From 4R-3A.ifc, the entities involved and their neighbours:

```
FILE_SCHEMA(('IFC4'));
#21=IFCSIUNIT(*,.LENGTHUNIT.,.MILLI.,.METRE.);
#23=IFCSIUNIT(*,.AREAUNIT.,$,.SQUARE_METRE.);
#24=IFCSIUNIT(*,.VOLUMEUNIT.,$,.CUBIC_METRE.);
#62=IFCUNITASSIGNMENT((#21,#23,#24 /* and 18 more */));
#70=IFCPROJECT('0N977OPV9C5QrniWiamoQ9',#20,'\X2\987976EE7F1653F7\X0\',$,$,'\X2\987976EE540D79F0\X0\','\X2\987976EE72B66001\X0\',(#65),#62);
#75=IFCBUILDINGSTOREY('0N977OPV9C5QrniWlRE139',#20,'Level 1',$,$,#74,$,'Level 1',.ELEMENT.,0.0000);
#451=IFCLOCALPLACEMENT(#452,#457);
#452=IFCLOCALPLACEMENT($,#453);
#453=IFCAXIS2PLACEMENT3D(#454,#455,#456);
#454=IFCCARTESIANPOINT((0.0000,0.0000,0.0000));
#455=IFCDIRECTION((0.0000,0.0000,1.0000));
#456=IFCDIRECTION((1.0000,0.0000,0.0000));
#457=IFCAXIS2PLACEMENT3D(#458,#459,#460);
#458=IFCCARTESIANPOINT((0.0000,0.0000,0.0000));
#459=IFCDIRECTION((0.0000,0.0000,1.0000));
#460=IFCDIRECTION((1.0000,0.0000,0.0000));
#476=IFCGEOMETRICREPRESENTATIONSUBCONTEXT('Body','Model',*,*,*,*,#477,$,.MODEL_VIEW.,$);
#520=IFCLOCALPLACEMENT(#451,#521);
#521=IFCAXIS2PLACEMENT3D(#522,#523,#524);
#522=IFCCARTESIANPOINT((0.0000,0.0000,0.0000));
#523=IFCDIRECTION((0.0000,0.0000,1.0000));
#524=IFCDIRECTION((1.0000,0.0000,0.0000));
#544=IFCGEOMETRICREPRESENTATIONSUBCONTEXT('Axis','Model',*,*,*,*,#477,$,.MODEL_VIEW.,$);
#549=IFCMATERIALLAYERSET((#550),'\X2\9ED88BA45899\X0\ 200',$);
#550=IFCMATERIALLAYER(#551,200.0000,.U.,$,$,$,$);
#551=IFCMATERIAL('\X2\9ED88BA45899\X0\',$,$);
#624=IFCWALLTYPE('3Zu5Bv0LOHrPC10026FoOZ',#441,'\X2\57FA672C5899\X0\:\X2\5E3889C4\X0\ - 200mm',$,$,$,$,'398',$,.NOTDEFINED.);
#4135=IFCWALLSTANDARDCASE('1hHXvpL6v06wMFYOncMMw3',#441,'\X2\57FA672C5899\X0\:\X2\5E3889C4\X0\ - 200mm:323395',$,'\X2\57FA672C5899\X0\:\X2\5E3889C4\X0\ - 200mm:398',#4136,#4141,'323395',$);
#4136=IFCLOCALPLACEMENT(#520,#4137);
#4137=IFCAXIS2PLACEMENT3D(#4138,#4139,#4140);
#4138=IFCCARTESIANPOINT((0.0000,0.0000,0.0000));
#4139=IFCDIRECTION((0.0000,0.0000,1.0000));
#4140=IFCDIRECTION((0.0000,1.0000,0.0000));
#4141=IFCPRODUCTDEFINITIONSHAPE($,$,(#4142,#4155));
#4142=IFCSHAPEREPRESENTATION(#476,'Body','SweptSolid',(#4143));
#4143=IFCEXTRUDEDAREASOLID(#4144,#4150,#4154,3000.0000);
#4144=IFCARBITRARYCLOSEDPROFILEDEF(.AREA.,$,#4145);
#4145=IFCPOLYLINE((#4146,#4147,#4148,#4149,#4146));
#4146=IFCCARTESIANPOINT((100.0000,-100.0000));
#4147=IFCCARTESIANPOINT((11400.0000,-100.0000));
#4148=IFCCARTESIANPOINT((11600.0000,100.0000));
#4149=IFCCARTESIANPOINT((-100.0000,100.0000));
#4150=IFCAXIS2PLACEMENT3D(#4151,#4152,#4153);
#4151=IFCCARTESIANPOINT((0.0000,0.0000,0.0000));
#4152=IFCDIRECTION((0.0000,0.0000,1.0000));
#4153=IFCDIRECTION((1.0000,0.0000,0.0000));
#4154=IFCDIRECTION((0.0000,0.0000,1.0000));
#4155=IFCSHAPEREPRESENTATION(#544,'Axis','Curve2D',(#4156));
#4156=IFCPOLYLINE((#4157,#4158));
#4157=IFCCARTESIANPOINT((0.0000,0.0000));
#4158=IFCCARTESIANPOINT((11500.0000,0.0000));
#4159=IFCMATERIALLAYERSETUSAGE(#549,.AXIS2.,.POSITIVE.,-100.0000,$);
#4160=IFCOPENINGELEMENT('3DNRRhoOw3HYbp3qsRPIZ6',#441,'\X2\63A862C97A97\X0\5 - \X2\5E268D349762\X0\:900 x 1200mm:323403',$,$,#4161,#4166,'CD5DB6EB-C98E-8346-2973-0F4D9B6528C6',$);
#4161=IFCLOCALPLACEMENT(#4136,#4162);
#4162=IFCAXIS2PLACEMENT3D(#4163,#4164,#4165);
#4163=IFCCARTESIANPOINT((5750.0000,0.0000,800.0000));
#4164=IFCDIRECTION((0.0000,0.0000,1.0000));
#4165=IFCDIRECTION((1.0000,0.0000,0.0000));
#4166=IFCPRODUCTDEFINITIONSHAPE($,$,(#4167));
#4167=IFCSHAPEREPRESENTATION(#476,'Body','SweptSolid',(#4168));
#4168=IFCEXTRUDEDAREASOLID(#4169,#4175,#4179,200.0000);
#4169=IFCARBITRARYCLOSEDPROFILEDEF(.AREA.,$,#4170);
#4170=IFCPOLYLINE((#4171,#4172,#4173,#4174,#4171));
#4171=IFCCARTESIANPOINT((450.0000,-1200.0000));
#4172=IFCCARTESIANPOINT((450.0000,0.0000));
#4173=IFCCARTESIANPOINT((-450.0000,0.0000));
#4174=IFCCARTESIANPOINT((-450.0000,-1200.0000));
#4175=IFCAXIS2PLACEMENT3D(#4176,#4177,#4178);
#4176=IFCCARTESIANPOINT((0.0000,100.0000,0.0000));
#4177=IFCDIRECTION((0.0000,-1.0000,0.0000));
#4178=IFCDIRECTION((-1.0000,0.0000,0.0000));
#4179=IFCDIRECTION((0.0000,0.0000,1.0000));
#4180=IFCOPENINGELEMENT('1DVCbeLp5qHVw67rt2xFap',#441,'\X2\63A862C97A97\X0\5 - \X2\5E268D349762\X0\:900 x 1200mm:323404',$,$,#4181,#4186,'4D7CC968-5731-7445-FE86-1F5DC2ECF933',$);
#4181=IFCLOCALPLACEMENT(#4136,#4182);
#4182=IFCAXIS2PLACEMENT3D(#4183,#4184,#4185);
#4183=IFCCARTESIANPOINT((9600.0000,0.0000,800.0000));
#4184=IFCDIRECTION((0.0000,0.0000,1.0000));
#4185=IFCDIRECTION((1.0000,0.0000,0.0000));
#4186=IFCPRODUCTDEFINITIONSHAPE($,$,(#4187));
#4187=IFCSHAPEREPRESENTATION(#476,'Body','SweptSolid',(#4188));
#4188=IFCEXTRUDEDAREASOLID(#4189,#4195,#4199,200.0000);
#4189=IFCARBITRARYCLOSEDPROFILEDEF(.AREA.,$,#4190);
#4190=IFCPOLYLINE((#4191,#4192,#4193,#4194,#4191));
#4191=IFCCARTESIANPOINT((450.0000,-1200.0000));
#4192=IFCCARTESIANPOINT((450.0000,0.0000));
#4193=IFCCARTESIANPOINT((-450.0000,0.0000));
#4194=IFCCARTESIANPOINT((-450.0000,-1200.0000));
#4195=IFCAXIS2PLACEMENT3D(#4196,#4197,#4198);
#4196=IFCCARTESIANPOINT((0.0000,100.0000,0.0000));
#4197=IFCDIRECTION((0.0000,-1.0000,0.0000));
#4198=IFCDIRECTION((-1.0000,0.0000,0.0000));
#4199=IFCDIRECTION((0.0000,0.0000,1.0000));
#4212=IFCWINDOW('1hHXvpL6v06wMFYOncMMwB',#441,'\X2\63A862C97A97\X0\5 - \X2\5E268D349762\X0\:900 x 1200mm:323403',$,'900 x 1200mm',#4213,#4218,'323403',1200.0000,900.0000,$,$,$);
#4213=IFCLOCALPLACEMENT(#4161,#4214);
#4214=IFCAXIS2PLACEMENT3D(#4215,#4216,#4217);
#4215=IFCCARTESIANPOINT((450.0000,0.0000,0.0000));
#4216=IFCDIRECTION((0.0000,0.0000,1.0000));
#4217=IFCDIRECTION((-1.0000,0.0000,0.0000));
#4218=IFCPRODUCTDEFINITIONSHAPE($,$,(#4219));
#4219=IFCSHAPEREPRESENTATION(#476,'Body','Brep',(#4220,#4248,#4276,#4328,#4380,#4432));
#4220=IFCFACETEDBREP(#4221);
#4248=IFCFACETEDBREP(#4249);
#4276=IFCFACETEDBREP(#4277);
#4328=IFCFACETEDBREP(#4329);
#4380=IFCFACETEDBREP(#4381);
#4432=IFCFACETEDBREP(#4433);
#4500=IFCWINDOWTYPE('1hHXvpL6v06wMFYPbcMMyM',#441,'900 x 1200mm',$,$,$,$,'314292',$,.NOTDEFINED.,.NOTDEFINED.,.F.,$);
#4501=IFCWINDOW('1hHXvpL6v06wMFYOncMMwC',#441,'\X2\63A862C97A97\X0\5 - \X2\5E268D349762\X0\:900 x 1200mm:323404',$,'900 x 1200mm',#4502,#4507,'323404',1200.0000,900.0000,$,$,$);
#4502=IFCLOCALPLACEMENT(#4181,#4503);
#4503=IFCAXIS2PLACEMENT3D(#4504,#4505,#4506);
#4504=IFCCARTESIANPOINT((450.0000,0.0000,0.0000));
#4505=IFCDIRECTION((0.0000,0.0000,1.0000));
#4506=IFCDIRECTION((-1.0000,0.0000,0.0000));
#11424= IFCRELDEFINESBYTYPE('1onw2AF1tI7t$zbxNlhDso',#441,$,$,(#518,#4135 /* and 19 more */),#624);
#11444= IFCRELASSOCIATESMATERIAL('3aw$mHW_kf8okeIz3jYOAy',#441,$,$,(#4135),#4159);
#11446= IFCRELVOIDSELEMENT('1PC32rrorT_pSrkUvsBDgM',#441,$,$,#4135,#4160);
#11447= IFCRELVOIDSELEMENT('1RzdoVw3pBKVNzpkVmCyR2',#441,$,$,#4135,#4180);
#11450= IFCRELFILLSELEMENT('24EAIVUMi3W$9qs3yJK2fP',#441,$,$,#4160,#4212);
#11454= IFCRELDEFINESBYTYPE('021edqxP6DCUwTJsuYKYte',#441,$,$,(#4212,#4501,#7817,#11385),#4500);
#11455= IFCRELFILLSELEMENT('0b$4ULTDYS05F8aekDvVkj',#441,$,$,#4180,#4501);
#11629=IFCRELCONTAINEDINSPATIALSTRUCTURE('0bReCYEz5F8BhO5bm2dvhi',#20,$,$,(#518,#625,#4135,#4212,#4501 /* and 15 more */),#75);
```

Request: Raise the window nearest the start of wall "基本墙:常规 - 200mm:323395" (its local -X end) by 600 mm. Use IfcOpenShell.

```python
import numpy as np
import ifcopenshell
import ifcopenshell.api.geometry
import ifcopenshell.util.placement
import ifcopenshell.util.unit

model = ifcopenshell.open("4R-3A.ifc")
unit_scale = ifcopenshell.util.unit.calculate_unit_scale(model)

window = model.by_guid("1hHXvpL6v06wMFYOncMMwB")
opening = window.FillsVoids[0].RelatingOpeningElement
dz = 0.6 / unit_scale

shift = np.array([0.0, 0.0, dz])
# The window is placed relative to its opening, so it follows when the opening moves.
matrix = ifcopenshell.util.placement.get_local_placement(opening.ObjectPlacement)
matrix[:3, 3] += shift
ifcopenshell.api.geometry.edit_object_placement(
    model, product=opening, matrix=matrix, is_si=False, should_transform_children=True
)

print(f"moved by {dz * unit_scale:+.3f} m")

model.write("4R-3A_updated.ifc")
```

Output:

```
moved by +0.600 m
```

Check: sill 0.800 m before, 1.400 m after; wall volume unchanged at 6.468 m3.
